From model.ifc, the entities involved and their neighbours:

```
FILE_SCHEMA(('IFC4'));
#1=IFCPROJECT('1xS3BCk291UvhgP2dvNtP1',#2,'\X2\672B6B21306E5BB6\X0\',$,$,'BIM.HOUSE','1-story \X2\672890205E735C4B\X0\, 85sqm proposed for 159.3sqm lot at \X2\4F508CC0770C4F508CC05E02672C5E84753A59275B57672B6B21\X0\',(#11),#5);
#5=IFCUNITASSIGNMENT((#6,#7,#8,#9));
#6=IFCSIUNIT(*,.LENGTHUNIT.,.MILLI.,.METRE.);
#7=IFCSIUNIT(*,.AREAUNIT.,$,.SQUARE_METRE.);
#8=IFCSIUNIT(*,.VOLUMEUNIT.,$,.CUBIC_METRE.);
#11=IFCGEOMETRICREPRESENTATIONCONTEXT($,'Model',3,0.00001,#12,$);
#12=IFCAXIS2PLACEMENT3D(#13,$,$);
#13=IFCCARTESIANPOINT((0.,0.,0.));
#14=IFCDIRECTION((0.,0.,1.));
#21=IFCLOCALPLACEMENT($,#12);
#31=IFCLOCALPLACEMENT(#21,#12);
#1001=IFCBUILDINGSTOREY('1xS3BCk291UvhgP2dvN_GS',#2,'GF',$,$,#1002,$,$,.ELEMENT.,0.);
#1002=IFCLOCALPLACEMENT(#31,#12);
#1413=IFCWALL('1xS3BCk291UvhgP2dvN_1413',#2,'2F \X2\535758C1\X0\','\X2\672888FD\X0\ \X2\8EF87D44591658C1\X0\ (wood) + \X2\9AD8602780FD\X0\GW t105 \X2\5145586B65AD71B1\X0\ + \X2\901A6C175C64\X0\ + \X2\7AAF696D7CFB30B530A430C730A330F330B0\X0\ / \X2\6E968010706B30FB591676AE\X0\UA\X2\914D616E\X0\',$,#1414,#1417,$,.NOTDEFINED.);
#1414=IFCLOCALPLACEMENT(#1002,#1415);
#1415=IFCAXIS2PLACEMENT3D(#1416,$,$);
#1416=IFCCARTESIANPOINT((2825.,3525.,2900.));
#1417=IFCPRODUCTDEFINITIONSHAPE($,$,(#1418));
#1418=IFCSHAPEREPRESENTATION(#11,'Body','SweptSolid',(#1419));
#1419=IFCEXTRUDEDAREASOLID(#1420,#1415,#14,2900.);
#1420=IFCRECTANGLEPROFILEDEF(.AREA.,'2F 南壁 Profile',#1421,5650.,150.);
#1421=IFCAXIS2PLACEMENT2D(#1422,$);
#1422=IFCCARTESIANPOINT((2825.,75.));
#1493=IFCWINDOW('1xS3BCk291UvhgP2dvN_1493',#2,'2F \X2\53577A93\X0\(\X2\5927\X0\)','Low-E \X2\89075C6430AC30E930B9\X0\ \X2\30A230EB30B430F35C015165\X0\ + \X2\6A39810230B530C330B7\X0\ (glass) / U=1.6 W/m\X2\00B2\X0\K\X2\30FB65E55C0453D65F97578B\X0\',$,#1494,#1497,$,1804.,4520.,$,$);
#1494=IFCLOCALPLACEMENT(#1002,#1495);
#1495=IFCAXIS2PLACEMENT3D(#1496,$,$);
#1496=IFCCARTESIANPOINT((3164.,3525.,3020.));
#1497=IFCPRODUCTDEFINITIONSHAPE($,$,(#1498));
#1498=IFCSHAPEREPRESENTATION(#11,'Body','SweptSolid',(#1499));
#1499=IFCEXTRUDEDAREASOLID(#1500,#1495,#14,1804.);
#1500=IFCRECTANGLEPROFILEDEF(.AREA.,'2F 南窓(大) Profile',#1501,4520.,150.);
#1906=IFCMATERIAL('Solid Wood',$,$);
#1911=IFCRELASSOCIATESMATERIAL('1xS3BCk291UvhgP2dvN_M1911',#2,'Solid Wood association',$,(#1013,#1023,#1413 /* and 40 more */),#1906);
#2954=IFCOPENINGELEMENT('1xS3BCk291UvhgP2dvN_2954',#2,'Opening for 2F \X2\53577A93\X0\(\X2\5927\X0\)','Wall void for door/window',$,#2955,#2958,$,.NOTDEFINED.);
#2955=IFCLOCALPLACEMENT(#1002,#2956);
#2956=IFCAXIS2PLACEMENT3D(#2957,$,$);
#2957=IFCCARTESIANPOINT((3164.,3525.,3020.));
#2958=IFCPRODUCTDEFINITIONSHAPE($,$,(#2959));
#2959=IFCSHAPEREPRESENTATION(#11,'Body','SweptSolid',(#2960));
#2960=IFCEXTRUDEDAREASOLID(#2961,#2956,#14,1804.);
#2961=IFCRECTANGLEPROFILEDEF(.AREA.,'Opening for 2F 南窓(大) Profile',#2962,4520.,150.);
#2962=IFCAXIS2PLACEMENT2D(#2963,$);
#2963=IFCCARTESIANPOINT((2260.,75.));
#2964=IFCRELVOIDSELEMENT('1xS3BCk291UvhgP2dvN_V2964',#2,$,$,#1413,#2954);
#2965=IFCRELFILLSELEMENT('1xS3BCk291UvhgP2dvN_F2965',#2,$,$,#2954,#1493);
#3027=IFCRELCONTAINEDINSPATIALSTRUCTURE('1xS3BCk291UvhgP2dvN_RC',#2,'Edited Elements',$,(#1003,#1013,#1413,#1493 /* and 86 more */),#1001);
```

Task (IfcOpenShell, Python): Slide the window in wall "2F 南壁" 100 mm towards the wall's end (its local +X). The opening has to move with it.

```python
import ifcopenshell
import ifcopenshell.api.geometry
import ifcopenshell.util.placement

model = ifcopenshell.open("model.ifc")

window = model.by_guid("1xS3BCk291UvhgP2dvN_1493")
opening = window.FillsVoids[0].RelatingOpeningElement
wall = opening.VoidsElements[0].RelatingBuildingElement

wall_matrix = ifcopenshell.util.placement.get_local_placement(wall.ObjectPlacement)
shift = wall_matrix[:3, 0] * 100.0
before = ifcopenshell.util.placement.get_local_placement(window.ObjectPlacement)[:3, 3].copy()

# The window is not placed relative to its opening, so move both.
for product in (opening, window):
    matrix = ifcopenshell.util.placement.get_local_placement(product.ObjectPlacement)
    matrix[:3, 3] += shift
    ifcopenshell.api.geometry.edit_object_placement(model, product=product, matrix=matrix, is_si=False)

after = ifcopenshell.util.placement.get_local_placement(window.ObjectPlacement)[:3, 3]
print("window moved by", (after - before).round(3) + 0.0)

model.write("model_edited.ifc")
```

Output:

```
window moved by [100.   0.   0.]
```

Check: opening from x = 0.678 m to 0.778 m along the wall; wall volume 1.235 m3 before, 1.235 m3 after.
